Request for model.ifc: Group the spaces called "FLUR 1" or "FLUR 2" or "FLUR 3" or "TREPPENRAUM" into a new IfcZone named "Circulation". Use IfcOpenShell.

First a look at what the model holds.

```python
import ifcopenshell

model = ifcopenshell.open("model.ifc")
print(model.schema)
seen = {}
for space in model.by_type("IfcSpace"):
    seen[space.LongName] = seen.get(space.LongName, 0) + 1
for name, count in sorted(seen.items(), key=str):
    print(count, "x", name)
print("zones:", [z.Name for z in model.by_type("IfcZone")][:20])
```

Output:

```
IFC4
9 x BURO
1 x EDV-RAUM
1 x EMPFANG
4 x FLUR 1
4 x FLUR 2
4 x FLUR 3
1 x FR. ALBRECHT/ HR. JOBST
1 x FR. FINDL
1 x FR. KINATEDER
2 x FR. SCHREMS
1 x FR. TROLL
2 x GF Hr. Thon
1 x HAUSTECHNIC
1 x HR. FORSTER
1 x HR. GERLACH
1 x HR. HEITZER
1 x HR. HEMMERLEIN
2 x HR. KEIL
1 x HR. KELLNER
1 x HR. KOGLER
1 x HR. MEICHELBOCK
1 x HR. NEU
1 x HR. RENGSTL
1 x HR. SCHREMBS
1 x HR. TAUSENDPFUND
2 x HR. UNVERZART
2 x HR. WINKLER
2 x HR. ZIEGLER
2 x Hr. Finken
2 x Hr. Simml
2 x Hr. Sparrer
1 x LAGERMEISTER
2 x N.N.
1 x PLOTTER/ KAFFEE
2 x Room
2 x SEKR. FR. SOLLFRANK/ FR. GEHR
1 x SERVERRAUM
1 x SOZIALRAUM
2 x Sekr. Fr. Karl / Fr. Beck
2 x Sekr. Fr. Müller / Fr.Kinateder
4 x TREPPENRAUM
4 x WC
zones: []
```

```python
import ifcopenshell
import ifcopenshell.api.group
import ifcopenshell.api.root

model = ifcopenshell.open("model.ifc")

names = {"FLUR 1", "FLUR 2", "FLUR 3", "TREPPENRAUM"}
spaces = [s for s in model.by_type("IfcSpace") if s.LongName in names]

zone = ifcopenshell.api.root.create_entity(model, ifc_class="IfcZone", name="Circulation")
ifcopenshell.api.group.assign_group(model, products=spaces, group=zone)
print(len(spaces), "spaces in", zone.Name)

model.write("model_rev.ifc")
```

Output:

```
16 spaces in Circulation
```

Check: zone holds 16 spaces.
